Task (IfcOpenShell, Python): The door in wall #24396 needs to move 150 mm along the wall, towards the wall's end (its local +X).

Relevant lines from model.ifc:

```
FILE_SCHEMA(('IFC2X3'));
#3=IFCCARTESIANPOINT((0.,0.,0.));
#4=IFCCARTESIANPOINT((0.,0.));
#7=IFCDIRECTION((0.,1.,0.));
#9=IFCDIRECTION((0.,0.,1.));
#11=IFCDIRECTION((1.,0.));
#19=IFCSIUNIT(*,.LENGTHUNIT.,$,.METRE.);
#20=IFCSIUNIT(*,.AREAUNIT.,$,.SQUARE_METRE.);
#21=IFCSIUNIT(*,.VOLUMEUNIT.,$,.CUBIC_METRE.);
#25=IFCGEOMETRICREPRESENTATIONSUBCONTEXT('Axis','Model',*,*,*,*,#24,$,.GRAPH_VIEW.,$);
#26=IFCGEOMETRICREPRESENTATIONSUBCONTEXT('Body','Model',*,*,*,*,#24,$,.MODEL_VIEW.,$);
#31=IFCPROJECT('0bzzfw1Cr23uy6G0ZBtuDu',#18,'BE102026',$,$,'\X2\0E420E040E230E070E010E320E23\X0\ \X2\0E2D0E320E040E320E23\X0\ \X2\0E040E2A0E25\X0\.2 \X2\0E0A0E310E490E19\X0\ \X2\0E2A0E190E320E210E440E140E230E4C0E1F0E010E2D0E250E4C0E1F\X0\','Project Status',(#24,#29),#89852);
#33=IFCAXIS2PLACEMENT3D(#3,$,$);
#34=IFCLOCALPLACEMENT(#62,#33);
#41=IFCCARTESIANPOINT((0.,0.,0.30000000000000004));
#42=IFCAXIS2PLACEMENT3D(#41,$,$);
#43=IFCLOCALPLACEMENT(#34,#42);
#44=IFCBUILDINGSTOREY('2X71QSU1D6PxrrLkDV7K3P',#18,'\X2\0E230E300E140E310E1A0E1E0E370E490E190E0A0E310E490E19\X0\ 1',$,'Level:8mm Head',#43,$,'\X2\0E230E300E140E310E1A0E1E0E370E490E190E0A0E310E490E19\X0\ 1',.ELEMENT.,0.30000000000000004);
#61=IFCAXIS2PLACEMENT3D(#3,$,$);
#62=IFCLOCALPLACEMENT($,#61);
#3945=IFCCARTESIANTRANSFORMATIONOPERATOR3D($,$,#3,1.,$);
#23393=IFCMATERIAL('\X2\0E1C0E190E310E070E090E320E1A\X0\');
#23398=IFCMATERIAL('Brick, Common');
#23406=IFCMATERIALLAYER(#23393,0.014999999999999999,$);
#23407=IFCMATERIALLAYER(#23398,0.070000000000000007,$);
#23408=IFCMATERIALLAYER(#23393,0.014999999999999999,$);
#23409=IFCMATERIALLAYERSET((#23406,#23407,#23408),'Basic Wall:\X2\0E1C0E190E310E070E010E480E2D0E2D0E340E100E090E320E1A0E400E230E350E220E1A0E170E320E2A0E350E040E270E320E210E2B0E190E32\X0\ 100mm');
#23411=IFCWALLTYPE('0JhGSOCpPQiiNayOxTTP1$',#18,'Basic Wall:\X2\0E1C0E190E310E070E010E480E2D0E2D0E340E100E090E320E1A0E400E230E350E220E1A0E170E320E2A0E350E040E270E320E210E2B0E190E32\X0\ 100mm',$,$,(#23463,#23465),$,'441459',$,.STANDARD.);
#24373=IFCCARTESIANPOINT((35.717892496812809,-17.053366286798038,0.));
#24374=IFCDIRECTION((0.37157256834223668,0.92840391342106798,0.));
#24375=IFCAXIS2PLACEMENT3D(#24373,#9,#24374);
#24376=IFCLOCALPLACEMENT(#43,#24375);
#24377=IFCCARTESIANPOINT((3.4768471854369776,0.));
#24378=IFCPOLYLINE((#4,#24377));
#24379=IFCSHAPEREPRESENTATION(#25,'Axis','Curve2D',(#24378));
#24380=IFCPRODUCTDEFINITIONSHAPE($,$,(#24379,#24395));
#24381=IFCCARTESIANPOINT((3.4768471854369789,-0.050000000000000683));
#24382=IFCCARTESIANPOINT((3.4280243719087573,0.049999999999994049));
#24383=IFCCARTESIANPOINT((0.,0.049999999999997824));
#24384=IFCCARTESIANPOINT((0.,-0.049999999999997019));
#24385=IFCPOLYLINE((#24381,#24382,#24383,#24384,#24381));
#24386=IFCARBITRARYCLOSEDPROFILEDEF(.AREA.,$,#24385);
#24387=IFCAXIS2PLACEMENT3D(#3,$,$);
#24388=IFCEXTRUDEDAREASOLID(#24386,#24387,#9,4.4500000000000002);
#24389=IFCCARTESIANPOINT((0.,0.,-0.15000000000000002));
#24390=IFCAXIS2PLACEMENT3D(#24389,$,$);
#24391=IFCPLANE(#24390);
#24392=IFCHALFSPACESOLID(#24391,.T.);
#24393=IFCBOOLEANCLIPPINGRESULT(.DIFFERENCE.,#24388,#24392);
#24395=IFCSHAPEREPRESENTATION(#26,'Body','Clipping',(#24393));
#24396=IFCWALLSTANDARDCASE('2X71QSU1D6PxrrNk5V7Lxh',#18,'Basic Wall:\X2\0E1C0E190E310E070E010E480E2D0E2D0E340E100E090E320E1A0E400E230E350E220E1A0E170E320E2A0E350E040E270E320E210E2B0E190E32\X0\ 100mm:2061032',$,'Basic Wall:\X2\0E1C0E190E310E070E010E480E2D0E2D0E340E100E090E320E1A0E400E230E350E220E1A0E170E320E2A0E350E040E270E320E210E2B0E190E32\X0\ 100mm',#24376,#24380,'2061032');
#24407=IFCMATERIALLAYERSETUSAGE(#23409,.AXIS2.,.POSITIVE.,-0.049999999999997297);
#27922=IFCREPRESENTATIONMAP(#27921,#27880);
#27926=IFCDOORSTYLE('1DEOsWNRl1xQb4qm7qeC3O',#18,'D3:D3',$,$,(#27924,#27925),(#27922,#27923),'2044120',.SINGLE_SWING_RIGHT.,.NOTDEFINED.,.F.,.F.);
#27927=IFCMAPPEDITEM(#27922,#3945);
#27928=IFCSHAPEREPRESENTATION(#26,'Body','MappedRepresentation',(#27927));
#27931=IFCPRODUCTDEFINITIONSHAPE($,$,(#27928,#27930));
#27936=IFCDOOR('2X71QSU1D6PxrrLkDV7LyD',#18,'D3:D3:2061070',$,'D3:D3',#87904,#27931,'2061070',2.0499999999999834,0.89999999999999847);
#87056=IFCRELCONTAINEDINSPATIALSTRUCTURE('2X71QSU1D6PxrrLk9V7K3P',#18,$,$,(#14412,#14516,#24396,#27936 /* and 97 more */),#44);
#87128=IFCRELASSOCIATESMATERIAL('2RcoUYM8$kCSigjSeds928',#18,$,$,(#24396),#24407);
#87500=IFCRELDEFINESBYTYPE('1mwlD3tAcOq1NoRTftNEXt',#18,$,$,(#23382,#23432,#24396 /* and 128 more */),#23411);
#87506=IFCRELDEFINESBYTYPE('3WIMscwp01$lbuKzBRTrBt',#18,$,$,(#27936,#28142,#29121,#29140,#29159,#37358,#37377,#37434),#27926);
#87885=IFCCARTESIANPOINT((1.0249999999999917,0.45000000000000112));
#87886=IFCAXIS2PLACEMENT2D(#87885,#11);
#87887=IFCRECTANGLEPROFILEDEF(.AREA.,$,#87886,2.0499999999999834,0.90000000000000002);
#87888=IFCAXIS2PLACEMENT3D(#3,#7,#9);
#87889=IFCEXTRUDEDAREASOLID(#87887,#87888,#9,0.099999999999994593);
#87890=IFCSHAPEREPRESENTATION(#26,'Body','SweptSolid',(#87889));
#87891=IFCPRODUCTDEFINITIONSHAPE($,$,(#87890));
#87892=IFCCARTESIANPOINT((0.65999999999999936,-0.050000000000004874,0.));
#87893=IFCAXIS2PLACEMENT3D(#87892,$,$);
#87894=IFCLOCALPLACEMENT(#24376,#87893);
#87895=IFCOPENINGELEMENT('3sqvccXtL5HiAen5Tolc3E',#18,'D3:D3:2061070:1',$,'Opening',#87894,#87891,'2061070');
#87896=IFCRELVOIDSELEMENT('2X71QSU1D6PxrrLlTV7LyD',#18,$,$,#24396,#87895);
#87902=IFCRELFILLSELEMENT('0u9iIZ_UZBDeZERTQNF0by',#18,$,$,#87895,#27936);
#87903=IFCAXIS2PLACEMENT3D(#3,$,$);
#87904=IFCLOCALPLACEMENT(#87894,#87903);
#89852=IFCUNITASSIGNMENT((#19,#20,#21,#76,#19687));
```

```python
import ifcopenshell
import ifcopenshell.api.geometry
import ifcopenshell.util.placement
import ifcopenshell.util.unit

model = ifcopenshell.open("model.ifc")
unit_scale = ifcopenshell.util.unit.calculate_unit_scale(model)

door = model.by_id(27936)
opening = door.FillsVoids[0].RelatingOpeningElement
wall = opening.VoidsElements[0].RelatingBuildingElement

wall_matrix = ifcopenshell.util.placement.get_local_placement(wall.ObjectPlacement)
shift = wall_matrix[:3, 0] * 0.15 / unit_scale
before = ifcopenshell.util.placement.get_local_placement(door.ObjectPlacement)[:3, 3].copy()

# The door is placed relative to its opening, so it follows when the opening moves.
matrix = ifcopenshell.util.placement.get_local_placement(opening.ObjectPlacement)
matrix[:3, 3] += shift
ifcopenshell.api.geometry.edit_object_placement(
    model, product=opening, matrix=matrix, is_si=False, should_transform_children=True
)

after = ifcopenshell.util.placement.get_local_placement(door.ObjectPlacement)[:3, 3]
print("door moved by", (after - before).round(3) + 0.0)

model.write("model-out.ifc")
```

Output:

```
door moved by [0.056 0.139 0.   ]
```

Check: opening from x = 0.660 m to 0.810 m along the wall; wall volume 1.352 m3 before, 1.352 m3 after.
